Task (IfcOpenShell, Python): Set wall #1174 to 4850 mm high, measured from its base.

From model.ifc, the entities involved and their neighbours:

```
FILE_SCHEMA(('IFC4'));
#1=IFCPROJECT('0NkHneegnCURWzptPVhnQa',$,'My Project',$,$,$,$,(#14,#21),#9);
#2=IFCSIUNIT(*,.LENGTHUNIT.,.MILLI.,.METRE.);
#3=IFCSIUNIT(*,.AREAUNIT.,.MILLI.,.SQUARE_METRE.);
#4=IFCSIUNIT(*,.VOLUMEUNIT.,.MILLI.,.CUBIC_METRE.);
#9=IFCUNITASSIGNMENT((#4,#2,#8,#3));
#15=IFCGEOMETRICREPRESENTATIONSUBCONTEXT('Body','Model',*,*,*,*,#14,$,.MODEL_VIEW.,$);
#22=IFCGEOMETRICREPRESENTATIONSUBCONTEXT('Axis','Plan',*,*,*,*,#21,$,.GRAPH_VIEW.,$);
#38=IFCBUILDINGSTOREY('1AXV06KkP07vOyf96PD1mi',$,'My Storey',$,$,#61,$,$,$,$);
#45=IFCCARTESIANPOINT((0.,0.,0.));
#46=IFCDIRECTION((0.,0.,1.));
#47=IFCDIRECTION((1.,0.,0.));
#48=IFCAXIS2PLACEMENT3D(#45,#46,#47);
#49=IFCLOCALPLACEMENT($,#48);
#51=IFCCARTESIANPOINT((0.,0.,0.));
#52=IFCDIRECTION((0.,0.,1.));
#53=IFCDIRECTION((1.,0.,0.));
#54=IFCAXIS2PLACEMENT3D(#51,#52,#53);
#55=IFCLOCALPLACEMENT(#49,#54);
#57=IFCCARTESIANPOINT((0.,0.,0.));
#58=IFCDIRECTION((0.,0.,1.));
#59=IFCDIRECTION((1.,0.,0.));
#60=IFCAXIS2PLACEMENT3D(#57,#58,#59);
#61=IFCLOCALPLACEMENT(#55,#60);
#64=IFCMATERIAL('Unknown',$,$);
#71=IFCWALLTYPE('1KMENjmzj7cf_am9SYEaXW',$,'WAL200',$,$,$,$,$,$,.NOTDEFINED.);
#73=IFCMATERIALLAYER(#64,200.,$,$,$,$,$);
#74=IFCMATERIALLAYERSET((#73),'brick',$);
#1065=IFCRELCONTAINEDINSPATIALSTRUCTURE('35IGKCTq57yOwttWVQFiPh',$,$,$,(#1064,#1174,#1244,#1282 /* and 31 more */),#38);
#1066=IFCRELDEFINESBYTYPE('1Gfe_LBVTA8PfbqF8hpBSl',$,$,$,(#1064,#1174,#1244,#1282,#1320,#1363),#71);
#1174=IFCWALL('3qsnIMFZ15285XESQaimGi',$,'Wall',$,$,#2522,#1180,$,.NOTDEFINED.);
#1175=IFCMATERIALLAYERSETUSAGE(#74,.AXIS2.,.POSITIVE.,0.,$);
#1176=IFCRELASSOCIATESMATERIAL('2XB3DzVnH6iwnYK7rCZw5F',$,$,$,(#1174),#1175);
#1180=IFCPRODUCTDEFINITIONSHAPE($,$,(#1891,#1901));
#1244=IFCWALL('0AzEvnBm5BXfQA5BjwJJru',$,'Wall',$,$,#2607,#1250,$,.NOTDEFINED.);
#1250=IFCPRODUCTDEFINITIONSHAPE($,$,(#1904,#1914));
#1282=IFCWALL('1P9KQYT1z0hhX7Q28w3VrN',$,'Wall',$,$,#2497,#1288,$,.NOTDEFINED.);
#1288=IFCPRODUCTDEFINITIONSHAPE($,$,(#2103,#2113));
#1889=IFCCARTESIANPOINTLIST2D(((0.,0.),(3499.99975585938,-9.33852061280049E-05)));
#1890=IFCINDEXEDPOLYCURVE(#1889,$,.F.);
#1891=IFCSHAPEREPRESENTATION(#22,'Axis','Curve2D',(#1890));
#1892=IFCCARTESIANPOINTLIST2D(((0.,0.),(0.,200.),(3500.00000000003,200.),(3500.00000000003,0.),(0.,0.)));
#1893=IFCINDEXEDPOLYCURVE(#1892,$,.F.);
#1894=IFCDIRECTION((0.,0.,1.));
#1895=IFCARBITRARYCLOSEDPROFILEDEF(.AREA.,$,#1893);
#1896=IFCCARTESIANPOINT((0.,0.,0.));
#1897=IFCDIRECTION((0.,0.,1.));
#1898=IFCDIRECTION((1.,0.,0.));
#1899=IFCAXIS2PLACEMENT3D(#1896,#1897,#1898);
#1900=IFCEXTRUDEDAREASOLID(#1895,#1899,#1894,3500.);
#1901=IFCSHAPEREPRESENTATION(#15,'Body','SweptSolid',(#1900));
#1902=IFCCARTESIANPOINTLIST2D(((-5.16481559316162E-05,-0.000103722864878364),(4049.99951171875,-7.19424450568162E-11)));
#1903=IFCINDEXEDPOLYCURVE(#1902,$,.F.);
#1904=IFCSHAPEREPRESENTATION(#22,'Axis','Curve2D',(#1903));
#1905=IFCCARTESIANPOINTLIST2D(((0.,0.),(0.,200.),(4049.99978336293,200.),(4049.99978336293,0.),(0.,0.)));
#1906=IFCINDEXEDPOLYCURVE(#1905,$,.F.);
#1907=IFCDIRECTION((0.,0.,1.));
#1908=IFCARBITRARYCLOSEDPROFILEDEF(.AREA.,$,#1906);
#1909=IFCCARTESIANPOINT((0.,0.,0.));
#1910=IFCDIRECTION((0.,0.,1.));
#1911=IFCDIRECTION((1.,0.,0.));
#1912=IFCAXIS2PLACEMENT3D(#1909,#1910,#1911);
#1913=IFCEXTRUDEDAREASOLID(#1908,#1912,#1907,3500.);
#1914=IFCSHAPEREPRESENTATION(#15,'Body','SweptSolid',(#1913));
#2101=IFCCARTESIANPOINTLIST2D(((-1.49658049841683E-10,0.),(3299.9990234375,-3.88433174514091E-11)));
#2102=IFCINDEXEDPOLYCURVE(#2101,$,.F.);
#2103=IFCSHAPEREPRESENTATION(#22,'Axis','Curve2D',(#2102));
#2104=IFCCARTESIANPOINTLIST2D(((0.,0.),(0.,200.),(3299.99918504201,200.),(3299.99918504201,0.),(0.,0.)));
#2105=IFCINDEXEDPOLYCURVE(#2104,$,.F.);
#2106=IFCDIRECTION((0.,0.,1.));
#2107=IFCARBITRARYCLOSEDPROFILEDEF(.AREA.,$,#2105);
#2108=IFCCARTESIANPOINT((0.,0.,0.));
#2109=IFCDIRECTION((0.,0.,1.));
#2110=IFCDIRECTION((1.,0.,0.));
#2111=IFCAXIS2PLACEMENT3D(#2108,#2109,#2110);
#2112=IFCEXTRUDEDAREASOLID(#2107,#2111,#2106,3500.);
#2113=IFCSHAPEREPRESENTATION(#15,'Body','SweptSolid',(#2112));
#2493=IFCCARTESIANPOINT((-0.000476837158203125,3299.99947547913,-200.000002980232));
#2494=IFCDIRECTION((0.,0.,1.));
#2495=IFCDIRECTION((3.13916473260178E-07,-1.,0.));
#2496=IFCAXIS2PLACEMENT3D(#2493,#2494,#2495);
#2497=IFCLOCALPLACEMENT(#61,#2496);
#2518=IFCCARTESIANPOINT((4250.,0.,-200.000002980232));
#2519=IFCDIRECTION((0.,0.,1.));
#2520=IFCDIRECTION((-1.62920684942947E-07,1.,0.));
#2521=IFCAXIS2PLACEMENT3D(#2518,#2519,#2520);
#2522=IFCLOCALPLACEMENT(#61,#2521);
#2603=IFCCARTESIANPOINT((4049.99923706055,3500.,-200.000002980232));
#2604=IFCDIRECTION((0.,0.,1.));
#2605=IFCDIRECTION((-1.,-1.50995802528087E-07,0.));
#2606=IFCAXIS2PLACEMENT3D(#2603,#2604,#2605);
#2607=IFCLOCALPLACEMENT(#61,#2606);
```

```python
import ifcopenshell
import ifcopenshell.geom
import ifcopenshell.util.representation
import ifcopenshell.util.shape
import ifcopenshell.util.unit

model = ifcopenshell.open("model.ifc")
unit_scale = ifcopenshell.util.unit.calculate_unit_scale(model)
settings = ifcopenshell.geom.settings()


def volume(element):
    """Net volume in cubic metres, openings subtracted."""
    shape = ifcopenshell.geom.create_shape(settings, element)
    return ifcopenshell.util.shape.get_volume(shape.geometry)


wall = model.by_id(1174)
before = volume(wall)

body = ifcopenshell.util.representation.get_representation(wall, "Model", "Body")
solid = body.Items[0]
old_height = solid.Depth
solid.Depth = 4.85 / unit_scale
after = volume(wall)

print(f"height {old_height:g} -> {solid.Depth:g}, volume {before:.3f} -> {after:.3f} m3")

model.write("model_rev.ifc")
```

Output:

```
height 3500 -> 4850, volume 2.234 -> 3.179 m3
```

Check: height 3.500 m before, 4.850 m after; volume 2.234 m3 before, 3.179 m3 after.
